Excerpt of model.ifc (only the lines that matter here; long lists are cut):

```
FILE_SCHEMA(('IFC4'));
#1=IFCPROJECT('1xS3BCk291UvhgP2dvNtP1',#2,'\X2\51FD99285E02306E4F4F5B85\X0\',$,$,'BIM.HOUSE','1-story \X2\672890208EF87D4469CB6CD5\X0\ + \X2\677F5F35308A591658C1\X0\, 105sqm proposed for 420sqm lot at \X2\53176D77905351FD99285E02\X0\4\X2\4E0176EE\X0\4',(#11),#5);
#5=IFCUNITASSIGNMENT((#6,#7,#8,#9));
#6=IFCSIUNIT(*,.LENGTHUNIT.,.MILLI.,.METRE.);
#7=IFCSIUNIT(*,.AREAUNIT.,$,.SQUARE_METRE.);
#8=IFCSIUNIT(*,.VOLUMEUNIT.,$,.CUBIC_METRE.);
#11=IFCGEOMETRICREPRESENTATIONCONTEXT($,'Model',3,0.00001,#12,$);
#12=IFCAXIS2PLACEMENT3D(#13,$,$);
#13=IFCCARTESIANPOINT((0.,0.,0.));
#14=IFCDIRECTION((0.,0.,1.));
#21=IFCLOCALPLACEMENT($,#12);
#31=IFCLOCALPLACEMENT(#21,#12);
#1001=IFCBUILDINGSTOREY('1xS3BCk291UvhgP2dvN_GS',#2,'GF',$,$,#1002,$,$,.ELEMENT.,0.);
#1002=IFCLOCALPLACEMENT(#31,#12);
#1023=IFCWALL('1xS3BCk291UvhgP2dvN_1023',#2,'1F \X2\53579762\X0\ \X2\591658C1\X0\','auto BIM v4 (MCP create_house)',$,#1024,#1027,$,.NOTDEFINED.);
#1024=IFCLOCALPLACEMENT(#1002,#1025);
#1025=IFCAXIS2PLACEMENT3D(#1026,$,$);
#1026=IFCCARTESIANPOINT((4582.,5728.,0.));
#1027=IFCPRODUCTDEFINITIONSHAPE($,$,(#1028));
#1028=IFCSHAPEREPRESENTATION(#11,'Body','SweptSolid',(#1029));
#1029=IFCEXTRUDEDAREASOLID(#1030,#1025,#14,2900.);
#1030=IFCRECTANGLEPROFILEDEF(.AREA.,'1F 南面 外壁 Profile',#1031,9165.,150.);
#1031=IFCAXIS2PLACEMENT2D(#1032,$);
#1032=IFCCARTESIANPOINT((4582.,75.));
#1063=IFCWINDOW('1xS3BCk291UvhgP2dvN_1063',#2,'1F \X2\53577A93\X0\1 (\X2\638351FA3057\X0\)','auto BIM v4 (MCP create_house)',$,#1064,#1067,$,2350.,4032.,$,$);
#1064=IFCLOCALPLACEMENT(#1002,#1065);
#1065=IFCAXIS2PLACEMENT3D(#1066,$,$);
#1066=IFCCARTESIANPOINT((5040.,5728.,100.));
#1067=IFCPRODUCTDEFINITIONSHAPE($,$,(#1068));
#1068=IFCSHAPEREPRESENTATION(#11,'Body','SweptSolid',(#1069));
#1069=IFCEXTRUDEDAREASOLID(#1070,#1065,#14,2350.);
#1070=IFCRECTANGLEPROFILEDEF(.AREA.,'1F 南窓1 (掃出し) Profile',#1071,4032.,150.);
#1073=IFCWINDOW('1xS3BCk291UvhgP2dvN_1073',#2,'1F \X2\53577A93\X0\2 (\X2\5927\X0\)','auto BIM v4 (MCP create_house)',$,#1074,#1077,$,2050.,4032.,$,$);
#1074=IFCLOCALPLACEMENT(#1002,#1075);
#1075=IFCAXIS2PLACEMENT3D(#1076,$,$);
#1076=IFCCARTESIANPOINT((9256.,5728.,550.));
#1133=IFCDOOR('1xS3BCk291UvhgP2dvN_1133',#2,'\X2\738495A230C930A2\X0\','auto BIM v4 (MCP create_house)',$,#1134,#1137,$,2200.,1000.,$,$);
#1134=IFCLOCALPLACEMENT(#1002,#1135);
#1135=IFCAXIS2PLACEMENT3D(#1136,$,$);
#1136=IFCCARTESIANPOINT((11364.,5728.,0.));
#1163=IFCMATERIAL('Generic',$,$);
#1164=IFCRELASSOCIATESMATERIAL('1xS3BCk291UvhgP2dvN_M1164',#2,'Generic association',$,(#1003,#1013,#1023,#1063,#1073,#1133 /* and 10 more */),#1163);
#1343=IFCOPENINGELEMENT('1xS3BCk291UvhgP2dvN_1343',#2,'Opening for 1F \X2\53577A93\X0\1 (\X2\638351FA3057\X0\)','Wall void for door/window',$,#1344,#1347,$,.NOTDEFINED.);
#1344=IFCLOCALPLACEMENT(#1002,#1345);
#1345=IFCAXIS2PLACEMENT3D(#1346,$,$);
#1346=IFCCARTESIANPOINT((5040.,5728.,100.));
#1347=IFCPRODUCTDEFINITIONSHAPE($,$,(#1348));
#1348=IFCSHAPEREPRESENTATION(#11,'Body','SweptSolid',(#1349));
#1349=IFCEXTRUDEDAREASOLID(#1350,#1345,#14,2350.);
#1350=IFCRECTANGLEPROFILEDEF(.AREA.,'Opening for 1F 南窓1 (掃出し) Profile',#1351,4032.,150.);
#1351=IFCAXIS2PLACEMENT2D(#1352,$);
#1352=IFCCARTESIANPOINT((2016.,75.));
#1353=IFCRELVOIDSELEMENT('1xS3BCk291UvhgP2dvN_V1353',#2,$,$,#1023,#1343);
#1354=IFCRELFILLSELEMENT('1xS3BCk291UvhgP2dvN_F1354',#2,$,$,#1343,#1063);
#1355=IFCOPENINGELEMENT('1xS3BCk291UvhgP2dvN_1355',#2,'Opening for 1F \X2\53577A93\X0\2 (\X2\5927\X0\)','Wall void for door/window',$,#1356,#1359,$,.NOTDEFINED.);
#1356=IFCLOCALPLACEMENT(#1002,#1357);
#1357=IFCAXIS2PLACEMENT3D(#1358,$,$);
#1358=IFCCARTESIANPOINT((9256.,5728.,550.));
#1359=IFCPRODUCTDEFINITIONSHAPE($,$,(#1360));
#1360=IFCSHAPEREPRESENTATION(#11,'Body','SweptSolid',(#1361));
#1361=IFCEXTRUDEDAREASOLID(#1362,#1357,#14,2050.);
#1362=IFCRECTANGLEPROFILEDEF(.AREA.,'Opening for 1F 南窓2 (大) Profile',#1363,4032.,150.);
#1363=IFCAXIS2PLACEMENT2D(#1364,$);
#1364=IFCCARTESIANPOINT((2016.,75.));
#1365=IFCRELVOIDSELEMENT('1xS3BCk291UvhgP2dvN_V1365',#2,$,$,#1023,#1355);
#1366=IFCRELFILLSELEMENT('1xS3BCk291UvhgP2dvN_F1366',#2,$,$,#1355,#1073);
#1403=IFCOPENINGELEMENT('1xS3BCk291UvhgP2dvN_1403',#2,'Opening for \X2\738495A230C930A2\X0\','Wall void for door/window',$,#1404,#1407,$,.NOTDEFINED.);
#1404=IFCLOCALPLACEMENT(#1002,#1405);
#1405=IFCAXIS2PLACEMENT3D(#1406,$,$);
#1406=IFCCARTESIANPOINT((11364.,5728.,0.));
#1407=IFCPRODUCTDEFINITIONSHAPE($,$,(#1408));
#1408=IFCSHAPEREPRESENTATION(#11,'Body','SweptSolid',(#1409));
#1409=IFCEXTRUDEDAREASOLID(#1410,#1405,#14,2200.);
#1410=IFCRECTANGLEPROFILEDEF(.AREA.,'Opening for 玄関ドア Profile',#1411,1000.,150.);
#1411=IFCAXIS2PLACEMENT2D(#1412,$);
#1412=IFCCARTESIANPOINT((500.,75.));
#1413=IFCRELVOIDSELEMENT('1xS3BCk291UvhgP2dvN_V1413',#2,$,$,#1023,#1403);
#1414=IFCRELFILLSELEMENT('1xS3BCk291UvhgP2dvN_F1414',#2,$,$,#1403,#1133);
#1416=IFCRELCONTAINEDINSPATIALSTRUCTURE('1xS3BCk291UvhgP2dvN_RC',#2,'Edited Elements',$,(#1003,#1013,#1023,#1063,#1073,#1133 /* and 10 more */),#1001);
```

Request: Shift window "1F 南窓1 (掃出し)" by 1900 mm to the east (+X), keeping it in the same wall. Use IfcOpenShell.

```python
import ifcopenshell
import ifcopenshell.api.geometry
import ifcopenshell.util.placement
import ifcopenshell.util.unit

model = ifcopenshell.open("model.ifc")
unit_scale = ifcopenshell.util.unit.calculate_unit_scale(model)

window = model.by_guid("1xS3BCk291UvhgP2dvN_1063")
opening = window.FillsVoids[0].RelatingOpeningElement
wall = opening.VoidsElements[0].RelatingBuildingElement

wall_matrix = ifcopenshell.util.placement.get_local_placement(wall.ObjectPlacement)
shift = wall_matrix[:3, 0] * 1.9 / unit_scale
before = ifcopenshell.util.placement.get_local_placement(window.ObjectPlacement)[:3, 3].copy()

# The window is not placed relative to its opening, so move both.
for product in (opening, window):
    matrix = ifcopenshell.util.placement.get_local_placement(product.ObjectPlacement)
    matrix[:3, 3] += shift
    ifcopenshell.api.geometry.edit_object_placement(model, product=product, matrix=matrix, is_si=False)

after = ifcopenshell.util.placement.get_local_placement(window.ObjectPlacement)[:3, 3]
print("window moved by", (after - before).round(3) + 0.0)

model.write("model_rev.ifc")
```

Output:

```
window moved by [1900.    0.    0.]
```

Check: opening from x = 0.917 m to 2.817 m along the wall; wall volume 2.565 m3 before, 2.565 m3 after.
